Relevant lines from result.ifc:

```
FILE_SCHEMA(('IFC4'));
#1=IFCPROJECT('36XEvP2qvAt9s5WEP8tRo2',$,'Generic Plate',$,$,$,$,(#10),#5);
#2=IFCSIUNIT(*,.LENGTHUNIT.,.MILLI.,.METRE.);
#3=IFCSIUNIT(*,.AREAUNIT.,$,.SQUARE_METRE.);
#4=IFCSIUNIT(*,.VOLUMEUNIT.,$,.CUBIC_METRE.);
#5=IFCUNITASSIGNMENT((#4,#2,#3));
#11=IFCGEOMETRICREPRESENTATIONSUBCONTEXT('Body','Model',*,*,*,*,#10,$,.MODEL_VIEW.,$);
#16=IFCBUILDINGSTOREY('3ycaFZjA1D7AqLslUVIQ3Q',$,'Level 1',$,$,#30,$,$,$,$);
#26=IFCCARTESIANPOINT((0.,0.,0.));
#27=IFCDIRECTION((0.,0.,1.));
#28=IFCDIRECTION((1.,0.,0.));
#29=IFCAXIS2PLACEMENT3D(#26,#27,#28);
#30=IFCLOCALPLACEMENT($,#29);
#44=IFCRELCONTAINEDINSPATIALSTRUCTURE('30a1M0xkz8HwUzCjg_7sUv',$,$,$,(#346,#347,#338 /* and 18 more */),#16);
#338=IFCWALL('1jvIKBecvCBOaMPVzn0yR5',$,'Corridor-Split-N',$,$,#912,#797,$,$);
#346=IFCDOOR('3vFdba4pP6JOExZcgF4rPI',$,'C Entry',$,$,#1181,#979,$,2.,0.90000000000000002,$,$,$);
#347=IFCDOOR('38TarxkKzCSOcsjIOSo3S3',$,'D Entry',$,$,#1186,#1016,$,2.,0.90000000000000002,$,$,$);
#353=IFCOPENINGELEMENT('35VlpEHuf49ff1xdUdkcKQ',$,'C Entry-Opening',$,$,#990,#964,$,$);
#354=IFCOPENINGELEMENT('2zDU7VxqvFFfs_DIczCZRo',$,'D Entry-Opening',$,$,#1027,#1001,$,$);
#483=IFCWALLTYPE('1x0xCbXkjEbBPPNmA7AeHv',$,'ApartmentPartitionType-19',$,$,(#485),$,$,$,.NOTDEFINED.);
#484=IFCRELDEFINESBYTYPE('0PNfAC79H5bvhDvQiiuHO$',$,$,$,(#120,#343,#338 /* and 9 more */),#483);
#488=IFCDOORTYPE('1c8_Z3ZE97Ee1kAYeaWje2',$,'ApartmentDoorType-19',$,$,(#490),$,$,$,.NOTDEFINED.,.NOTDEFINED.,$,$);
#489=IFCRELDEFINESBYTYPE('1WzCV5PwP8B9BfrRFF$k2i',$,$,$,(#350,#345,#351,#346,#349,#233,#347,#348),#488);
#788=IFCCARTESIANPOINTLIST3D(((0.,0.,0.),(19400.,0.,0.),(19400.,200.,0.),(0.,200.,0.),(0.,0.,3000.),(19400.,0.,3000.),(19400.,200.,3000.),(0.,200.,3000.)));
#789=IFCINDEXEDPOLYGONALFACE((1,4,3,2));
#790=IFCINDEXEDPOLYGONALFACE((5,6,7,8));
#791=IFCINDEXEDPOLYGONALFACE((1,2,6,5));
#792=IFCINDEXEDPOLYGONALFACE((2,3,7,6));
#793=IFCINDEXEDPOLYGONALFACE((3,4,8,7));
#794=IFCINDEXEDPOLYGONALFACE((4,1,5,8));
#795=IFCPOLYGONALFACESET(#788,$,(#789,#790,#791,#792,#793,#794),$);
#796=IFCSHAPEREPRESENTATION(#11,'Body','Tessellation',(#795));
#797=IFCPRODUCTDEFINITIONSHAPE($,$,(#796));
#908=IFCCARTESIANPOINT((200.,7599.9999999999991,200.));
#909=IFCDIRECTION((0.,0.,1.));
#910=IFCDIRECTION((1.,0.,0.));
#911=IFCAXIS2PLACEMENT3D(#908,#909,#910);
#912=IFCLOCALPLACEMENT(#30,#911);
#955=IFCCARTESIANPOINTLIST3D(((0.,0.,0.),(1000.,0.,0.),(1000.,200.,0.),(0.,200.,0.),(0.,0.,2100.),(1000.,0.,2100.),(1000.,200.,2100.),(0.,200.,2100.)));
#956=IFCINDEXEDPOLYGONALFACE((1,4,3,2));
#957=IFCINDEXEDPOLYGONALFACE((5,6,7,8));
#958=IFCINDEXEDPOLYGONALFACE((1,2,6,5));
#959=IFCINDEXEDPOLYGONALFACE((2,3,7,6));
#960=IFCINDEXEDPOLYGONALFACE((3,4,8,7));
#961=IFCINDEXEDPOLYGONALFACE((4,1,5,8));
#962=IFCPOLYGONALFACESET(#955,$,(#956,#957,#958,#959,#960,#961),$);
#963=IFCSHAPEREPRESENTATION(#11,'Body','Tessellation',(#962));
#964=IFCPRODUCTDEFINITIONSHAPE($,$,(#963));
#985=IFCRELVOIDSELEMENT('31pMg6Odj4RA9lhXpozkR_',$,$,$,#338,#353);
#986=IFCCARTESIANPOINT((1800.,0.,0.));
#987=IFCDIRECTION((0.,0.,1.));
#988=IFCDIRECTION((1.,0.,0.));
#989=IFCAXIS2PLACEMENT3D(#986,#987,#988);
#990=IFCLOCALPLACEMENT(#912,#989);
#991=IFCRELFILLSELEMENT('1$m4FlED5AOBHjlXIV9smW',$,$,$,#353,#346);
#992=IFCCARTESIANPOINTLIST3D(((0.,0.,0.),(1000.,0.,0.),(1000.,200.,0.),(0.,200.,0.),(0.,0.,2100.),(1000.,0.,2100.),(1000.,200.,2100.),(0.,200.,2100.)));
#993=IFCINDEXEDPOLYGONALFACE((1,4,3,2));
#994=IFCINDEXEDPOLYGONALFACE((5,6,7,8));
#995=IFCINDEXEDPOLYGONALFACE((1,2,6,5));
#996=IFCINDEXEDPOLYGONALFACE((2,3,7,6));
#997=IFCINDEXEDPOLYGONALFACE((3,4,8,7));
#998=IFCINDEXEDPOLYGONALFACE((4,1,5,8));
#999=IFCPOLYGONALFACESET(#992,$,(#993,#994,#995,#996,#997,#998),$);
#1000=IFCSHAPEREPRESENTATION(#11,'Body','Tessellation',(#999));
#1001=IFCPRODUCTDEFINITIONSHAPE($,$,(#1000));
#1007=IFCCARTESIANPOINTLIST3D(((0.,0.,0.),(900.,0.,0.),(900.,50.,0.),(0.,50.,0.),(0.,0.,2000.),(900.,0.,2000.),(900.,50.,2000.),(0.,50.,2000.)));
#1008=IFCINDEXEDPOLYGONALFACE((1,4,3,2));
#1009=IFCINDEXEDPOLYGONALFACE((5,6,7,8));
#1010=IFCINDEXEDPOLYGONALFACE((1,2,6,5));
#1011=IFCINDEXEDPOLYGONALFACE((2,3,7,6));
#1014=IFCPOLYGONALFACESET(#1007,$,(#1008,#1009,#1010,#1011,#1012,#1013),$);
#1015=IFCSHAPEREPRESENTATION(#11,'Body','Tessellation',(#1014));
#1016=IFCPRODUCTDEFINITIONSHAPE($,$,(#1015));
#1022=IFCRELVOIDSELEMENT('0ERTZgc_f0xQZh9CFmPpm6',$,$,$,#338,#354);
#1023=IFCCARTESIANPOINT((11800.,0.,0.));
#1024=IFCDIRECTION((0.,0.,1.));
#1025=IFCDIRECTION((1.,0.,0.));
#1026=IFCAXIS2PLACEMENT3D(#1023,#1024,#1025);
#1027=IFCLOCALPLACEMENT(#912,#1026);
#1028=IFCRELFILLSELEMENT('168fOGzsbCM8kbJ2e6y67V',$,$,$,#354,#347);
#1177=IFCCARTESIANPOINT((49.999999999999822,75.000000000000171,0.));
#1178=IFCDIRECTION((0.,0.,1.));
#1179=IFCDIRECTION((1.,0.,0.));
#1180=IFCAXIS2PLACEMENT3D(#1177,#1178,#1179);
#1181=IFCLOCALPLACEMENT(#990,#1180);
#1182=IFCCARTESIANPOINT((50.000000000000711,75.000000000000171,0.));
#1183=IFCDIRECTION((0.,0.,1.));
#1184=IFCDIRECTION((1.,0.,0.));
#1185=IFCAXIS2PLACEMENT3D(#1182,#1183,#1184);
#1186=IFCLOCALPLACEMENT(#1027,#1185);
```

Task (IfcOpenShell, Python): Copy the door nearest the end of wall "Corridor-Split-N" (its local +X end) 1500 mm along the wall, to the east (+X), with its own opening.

```python
import ifcopenshell
import ifcopenshell.api.feature
import ifcopenshell.api.geometry
import ifcopenshell.api.root
import ifcopenshell.geom
import ifcopenshell.util.element
import ifcopenshell.util.placement
import ifcopenshell.util.shape

model = ifcopenshell.open("result.ifc")
settings = ifcopenshell.geom.settings()


def volume(element):
    """Net volume in cubic metres, openings subtracted."""
    shape = ifcopenshell.geom.create_shape(settings, element)
    return ifcopenshell.util.shape.get_volume(shape.geometry)


door = model.by_guid("38TarxkKzCSOcsjIOSo3S3")
opening = door.FillsVoids[0].RelatingOpeningElement
wall = opening.VoidsElements[0].RelatingBuildingElement
before = volume(wall)
shift = ifcopenshell.util.placement.get_local_placement(wall.ObjectPlacement)[:3, 0] * 1500.0

# copy_class copies the void relationship, type, container and properties, but no geometry.
new_opening = ifcopenshell.api.root.copy_class(model, product=opening)
new_opening.Representation = ifcopenshell.util.element.copy_deep(
    model, opening.Representation, exclude=["IfcGeometricRepresentationContext", "IfcRepresentationMap"]
)
new_door = ifcopenshell.api.root.copy_class(model, product=door)
new_door.Representation = ifcopenshell.util.element.copy_deep(
    model, door.Representation, exclude=["IfcGeometricRepresentationContext", "IfcRepresentationMap"]
)
ifcopenshell.api.feature.add_filling(model, opening=new_opening, element=new_door)

for old, new in ((opening, new_opening), (door, new_door)):
    matrix = ifcopenshell.util.placement.get_local_placement(old.ObjectPlacement)
    matrix[:3, 3] += shift
    ifcopenshell.api.geometry.edit_object_placement(model, product=new, matrix=matrix, is_si=False)

after = volume(wall)

print(f"wall volume {before:.3f} -> {after:.3f} m3")

model.write("result_updated.ifc")
```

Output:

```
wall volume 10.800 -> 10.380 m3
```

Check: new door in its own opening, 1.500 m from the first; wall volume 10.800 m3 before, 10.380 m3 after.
